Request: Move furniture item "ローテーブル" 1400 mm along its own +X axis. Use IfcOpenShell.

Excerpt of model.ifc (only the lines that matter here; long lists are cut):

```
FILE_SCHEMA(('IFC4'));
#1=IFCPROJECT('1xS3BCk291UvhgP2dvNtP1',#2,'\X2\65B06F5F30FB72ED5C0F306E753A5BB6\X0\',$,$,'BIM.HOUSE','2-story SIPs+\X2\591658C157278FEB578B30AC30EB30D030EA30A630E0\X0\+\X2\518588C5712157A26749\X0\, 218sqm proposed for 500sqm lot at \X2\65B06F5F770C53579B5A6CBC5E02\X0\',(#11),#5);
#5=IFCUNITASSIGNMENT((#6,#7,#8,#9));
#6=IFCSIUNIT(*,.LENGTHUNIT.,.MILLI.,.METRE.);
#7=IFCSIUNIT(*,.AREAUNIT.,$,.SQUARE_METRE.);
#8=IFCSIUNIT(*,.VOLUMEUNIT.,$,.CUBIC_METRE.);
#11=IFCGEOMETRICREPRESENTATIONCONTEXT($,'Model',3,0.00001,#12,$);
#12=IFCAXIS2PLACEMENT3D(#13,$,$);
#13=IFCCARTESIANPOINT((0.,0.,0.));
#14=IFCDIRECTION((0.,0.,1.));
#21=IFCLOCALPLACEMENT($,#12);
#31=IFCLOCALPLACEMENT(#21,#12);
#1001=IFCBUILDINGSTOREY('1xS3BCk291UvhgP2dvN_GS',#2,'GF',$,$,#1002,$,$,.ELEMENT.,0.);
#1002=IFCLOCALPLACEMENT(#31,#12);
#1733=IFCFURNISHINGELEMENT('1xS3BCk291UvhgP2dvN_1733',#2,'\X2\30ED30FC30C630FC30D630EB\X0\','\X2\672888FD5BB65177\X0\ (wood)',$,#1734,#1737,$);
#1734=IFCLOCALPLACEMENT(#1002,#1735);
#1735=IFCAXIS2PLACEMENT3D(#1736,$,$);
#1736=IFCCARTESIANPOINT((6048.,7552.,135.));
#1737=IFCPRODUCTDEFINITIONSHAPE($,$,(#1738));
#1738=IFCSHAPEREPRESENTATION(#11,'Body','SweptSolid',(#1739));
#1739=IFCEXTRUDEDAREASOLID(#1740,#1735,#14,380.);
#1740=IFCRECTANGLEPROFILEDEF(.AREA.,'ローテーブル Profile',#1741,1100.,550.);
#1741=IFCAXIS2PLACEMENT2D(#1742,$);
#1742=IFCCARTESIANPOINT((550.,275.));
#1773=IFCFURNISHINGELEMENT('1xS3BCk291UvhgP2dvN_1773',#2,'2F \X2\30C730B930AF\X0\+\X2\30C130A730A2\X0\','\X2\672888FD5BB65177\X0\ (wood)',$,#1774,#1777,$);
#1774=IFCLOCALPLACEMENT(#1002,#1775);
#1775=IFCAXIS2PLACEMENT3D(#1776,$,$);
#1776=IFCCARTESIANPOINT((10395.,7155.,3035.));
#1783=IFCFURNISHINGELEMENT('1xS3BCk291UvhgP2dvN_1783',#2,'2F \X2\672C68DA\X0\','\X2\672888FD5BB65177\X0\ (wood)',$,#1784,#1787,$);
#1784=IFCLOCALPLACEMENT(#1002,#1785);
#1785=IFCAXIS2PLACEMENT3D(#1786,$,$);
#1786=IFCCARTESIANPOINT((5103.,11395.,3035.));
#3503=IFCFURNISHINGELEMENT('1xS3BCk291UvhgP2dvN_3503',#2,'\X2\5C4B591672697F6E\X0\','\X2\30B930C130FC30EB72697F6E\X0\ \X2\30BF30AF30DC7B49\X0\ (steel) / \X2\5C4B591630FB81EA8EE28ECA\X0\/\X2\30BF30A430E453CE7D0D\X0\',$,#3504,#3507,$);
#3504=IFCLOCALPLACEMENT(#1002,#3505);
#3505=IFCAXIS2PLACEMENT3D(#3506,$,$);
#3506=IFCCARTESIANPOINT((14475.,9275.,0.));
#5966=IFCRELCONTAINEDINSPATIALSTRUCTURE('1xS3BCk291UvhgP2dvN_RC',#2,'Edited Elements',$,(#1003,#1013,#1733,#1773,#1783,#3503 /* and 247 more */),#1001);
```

```python
import ifcopenshell
import ifcopenshell.api.geometry
import ifcopenshell.util.placement
import ifcopenshell.util.unit

model = ifcopenshell.open("model.ifc")
unit_scale = ifcopenshell.util.unit.calculate_unit_scale(model)

item = model.by_id(1733)
matrix = ifcopenshell.util.placement.get_local_placement(item.ObjectPlacement)
matrix[:3, 3] += matrix[:3, 0] * 1.4 / unit_scale
ifcopenshell.api.geometry.edit_object_placement(model, product=item, matrix=matrix, is_si=False)

print(ifcopenshell.util.placement.get_local_placement(item.ObjectPlacement).round(3) + 0.0)

model.write("model_rev.ifc")
```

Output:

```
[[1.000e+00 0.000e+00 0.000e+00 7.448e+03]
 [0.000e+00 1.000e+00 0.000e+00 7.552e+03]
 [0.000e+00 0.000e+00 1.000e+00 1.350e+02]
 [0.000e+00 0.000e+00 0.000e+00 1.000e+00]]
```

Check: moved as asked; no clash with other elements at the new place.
